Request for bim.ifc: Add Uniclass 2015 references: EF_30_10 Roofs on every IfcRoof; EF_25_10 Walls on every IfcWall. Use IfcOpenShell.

First a look at what the model holds.

```python
import ifcopenshell

model = ifcopenshell.open("bim.ifc")
print(model.schema)
print("classifications:", [c.Name for c in model.by_type("IfcClassification")])
for ifc_class in ("IfcDoor", "IfcRoof", "IfcStair", "IfcWall", "IfcWindow"):
    print(ifc_class, len(model.by_type(ifc_class)))
```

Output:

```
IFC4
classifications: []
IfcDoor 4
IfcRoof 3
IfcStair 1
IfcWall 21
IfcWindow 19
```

```python
import ifcopenshell
import ifcopenshell.api.classification

model = ifcopenshell.open("bim.ifc")

system = ifcopenshell.api.classification.add_classification(model, classification="Uniclass 2015")

codes = {
    "IfcRoof": ("EF_30_10", "Roofs"),
    "IfcWall": ("EF_25_10", "Walls"),
}
for ifc_class, (code, name) in codes.items():
    products = model.by_type(ifc_class)
    ifcopenshell.api.classification.add_reference(
        model, products=products, classification=system, identification=code, name=name
    )
    print(code, len(products))

model.write("bim_v2.ifc")
```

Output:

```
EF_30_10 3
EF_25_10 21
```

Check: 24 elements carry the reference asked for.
